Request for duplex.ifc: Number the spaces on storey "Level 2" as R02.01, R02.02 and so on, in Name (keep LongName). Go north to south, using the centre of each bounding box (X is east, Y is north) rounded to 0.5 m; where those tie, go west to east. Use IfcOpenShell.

First a look at what the model holds.

```python
import ifcopenshell
import ifcopenshell.util.element
import ifcopenshell.util.placement

model = ifcopenshell.open("duplex.ifc")
print(model.schema)
storey = next(s for s in model.by_type("IfcBuildingStorey") if s.Name == "Level 2")
spaces = [e for e in ifcopenshell.util.element.get_decomposition(storey) if e.is_a("IfcSpace")]
for e in sorted(spaces, key=lambda e: e.id()):
    origin = ifcopenshell.util.placement.get_local_placement(e.ObjectPlacement)[:3, 3]
    print(e.id(), e.Name, e.LongName, origin.round(2) + 0.0, sep=" | ")
```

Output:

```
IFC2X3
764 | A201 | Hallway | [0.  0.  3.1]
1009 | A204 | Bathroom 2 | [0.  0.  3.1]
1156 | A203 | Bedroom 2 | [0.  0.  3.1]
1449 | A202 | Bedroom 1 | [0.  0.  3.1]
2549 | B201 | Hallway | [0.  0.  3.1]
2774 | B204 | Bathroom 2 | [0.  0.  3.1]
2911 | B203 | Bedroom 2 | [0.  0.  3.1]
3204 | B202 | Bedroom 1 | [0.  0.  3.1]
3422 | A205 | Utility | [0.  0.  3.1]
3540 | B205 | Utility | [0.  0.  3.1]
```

```python
import ifcopenshell
import ifcopenshell.geom
import ifcopenshell.util.element
import ifcopenshell.util.shape

model = ifcopenshell.open("duplex.ifc")
settings = ifcopenshell.geom.settings()
settings.set("use-world-coords", True)


def centre(element):
    shape = ifcopenshell.geom.create_shape(settings, element)
    return ifcopenshell.util.shape.get_bbox_centroid(shape.geometry)


storey = next(s for s in model.by_type("IfcBuildingStorey") if s.Name == "Level 2")
spaces = [e for e in ifcopenshell.util.element.get_decomposition(storey) if e.is_a("IfcSpace")]

# Insertion points can sit at a corner or the storey origin, so sort by the geometry (in metres).
centres = {e: centre(e) for e in spaces}
spaces.sort(key=lambda e: (-round(centres[e][1] / 0.5), centres[e][0]))

for i, e in enumerate(spaces, start=1):
    number = f"R02.{i:02d}"
    e.Name = number
    print(e.id(), number)

model.write("duplex_updated.ifc")
```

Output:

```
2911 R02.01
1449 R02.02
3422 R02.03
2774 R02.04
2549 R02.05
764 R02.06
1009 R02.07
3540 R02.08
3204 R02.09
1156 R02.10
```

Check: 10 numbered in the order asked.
